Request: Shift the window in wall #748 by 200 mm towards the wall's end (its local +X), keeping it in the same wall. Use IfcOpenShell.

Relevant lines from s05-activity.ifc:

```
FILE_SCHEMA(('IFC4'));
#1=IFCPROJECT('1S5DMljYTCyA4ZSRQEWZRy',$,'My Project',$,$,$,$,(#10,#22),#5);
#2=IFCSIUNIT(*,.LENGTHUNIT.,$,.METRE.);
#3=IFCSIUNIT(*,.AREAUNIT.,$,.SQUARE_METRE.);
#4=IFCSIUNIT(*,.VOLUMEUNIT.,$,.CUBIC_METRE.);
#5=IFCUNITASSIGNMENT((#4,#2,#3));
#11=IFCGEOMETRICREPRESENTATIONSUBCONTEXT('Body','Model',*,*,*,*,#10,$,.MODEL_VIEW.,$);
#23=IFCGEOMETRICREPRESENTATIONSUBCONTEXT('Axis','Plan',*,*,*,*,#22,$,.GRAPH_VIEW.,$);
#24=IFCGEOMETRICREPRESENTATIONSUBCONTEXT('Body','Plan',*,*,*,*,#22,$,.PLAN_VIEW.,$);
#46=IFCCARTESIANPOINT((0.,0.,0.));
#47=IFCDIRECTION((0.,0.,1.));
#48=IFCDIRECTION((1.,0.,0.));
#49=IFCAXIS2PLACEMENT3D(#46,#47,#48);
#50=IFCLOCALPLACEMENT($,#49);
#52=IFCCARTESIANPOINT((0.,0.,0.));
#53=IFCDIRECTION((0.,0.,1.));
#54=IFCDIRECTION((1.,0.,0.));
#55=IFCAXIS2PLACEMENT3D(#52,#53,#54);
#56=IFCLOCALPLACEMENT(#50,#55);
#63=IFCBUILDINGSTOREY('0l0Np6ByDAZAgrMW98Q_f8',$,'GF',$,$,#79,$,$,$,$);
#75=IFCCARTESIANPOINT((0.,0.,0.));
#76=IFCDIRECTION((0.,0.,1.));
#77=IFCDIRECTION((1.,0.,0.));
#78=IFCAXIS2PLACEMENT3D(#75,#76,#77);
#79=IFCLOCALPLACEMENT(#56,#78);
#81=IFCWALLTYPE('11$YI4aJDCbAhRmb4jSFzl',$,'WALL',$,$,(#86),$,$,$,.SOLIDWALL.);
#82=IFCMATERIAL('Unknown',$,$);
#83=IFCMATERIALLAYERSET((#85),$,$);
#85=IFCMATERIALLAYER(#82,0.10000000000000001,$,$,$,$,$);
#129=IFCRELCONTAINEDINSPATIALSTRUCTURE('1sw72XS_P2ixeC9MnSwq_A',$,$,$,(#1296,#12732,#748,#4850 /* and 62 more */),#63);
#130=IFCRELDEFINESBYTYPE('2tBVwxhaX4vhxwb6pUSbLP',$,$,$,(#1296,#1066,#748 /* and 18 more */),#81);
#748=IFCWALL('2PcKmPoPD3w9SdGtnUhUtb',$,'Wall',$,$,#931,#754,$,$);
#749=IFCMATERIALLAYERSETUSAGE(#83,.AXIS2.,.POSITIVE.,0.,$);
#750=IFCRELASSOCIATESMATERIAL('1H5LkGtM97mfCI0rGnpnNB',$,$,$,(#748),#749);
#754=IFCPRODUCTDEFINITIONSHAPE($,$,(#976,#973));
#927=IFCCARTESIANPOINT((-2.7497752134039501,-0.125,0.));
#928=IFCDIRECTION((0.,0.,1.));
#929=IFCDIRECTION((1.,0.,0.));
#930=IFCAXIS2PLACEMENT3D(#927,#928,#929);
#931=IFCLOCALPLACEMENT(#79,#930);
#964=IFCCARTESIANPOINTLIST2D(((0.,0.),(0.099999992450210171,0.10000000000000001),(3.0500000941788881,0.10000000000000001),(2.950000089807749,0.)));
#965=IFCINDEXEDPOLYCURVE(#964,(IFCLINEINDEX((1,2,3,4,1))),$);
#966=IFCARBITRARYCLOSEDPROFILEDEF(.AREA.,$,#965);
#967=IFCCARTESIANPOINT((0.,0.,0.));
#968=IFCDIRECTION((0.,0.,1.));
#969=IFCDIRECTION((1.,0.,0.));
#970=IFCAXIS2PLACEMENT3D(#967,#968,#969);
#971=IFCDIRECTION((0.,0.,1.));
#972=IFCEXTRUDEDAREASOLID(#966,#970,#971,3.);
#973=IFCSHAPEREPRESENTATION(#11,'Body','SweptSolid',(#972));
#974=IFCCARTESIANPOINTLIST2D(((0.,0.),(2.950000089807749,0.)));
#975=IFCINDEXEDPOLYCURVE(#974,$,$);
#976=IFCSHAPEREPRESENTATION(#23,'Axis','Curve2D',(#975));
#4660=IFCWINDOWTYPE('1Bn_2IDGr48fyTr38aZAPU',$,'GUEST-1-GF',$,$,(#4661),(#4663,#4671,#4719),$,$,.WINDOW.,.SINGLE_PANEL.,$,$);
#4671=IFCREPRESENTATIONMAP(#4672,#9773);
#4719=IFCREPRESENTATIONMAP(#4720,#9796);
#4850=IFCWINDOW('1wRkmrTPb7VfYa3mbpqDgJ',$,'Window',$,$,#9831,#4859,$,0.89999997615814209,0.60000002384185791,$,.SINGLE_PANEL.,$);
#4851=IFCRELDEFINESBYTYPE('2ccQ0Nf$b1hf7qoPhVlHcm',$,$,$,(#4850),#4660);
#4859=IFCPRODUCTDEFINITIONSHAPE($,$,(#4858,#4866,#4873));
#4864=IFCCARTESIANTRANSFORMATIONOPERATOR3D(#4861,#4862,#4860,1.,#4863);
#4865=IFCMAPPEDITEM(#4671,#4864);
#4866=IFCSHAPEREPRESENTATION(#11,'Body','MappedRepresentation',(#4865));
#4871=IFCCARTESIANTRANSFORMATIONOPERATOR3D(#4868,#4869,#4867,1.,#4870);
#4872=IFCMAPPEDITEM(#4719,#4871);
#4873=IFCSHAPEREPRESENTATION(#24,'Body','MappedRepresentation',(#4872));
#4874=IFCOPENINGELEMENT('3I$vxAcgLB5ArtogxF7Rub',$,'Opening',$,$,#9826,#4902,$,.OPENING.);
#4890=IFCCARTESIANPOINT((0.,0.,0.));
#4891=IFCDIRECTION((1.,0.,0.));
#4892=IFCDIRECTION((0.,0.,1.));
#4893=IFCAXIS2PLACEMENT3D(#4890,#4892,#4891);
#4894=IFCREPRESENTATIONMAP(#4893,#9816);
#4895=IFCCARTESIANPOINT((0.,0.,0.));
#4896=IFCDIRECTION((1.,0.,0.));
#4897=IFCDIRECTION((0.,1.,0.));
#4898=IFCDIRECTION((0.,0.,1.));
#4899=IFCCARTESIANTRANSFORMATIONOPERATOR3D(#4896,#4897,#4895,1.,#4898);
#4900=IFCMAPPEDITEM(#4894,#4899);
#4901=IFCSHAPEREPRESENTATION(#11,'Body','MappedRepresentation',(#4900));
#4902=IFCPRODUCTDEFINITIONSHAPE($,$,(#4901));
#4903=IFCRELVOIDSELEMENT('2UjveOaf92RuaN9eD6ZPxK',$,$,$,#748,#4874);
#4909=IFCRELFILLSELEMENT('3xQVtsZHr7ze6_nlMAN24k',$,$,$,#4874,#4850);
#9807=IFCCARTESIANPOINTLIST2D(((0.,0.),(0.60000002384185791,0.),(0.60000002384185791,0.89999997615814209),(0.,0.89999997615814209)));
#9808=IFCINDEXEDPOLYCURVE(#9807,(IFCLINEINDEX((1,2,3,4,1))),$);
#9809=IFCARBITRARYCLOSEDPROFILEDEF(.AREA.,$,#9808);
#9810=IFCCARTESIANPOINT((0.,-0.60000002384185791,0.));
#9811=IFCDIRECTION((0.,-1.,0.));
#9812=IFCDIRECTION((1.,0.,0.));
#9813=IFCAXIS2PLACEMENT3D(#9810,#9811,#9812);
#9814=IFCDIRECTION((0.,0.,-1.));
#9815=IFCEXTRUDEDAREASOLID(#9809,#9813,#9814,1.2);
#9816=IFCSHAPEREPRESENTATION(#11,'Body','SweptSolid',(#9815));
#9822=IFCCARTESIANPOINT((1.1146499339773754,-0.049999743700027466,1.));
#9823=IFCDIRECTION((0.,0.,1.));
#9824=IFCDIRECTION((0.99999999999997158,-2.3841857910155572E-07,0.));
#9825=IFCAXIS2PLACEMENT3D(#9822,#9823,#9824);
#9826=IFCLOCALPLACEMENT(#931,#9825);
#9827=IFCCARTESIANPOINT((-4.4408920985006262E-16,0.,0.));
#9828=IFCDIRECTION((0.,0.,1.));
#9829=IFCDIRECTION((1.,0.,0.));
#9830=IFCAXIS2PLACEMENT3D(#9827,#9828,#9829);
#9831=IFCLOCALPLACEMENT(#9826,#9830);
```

```python
import ifcopenshell
import ifcopenshell.api.geometry
import ifcopenshell.util.placement
import ifcopenshell.util.unit

model = ifcopenshell.open("s05-activity.ifc")
unit_scale = ifcopenshell.util.unit.calculate_unit_scale(model)

window = model.by_id(4850)
opening = window.FillsVoids[0].RelatingOpeningElement
wall = opening.VoidsElements[0].RelatingBuildingElement

wall_matrix = ifcopenshell.util.placement.get_local_placement(wall.ObjectPlacement)
shift = wall_matrix[:3, 0] * 0.2 / unit_scale
before = ifcopenshell.util.placement.get_local_placement(window.ObjectPlacement)[:3, 3].copy()

# The window is placed relative to its opening, so it follows when the opening moves.
matrix = ifcopenshell.util.placement.get_local_placement(opening.ObjectPlacement)
matrix[:3, 3] += shift
ifcopenshell.api.geometry.edit_object_placement(
    model, product=opening, matrix=matrix, is_si=False, should_transform_children=True
)

after = ifcopenshell.util.placement.get_local_placement(window.ObjectPlacement)[:3, 3]
print("window moved by", (after - before).round(3) + 0.0)

model.write("s05-activity_edited.ifc")
```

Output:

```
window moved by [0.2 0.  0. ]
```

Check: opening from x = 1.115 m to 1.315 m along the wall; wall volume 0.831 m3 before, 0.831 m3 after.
